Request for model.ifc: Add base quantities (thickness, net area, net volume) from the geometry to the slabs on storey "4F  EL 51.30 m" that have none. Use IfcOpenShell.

First a look at what the model holds.

```python
import ifcopenshell
import ifcopenshell.util.element
import ifcopenshell.util.unit

model = ifcopenshell.open("model.ifc")
print(model.schema)
for unit_type in ("LENGTHUNIT", "AREAUNIT", "VOLUMEUNIT"):
    print(unit_type, ifcopenshell.util.unit.calculate_unit_scale(model, unit_type))
storey = next(s for s in model.by_type("IfcBuildingStorey") if s.Name == "4F  EL 51.30 m")
slabs = [e for e in ifcopenshell.util.element.get_decomposition(storey) if e.is_a("IfcSlab")]
for e in sorted(slabs, key=lambda e: e.id()):
    print(e.id(), e.is_a(), e.Name, list(ifcopenshell.util.element.get_psets(e, qtos_only=True)), sep=" | ")
```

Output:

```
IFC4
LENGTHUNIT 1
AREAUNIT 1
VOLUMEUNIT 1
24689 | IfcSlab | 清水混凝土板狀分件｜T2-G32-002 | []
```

```python
import ifcopenshell
import ifcopenshell.api.pset
import ifcopenshell.geom
import ifcopenshell.util.element
import ifcopenshell.util.shape
import ifcopenshell.util.unit

model = ifcopenshell.open("model.ifc")
unit_scale = ifcopenshell.util.unit.calculate_unit_scale(model)
area_scale = ifcopenshell.util.unit.calculate_unit_scale(model, "AREAUNIT")
volume_scale = ifcopenshell.util.unit.calculate_unit_scale(model, "VOLUMEUNIT")
settings = ifcopenshell.geom.settings()

storey = next(s for s in model.by_type("IfcBuildingStorey") if s.Name == "4F  EL 51.30 m")
slabs = [e for e in ifcopenshell.util.element.get_decomposition(storey) if e.is_a("IfcSlab")]

for e in sorted(slabs, key=lambda e: e.id()):
    if ifcopenshell.util.element.get_psets(e, qtos_only=True, should_inherit=False):
        continue
    # Geometry comes back in metres, in the element's own axes.
    shape = ifcopenshell.geom.create_shape(settings, e)
    values = {
        "Width": ifcopenshell.util.shape.get_z(shape.geometry) / unit_scale,
        "NetArea": ifcopenshell.util.shape.get_footprint_area(shape.geometry) / area_scale,
        "NetVolume": ifcopenshell.util.shape.get_volume(shape.geometry) / volume_scale,
    }
    qto = ifcopenshell.api.pset.add_qto(model, product=e, name="Qto_SlabBaseQuantities")
    ifcopenshell.api.pset.edit_qto(model, qto=qto, properties=values)
    print(e.id(), {k: round(v, 3) for k, v in values.items()})

model.write("model_rev.ifc")
```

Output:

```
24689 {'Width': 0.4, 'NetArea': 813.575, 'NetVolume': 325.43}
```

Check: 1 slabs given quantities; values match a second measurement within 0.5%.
